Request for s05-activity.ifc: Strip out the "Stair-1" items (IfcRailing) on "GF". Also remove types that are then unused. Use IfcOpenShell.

First a look at what the model holds.

```python
import ifcopenshell
import ifcopenshell.util.element

model = ifcopenshell.open("s05-activity.ifc")
print(model.schema)
storey = next(s for s in model.by_type("IfcBuildingStorey") if s.Name == "GF")
railings = [e for e in ifcopenshell.util.element.get_decomposition(storey) if e.is_a("IfcRailing")]
seen = {}
for e in railings:
    element_type = ifcopenshell.util.element.get_type(e)
    name = element_type.Name if element_type not in (None, e) else None
    seen[name] = seen.get(name, 0) + 1
for name, count in sorted(seen.items(), key=str):
    print(count, "x", name)
```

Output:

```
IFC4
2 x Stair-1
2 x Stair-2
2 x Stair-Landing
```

```python
import ifcopenshell
import ifcopenshell.api.root
import ifcopenshell.util.element

model = ifcopenshell.open("s05-activity.ifc")

storey = next(s for s in model.by_type("IfcBuildingStorey") if s.Name == "GF")
railings = [e for e in ifcopenshell.util.element.get_decomposition(storey) if e.is_a("IfcRailing")]
targets = [e for e in railings if (t := ifcopenshell.util.element.get_type(e)) not in (None, e) and t.Name == "Stair-1"]
types = {ifcopenshell.util.element.get_type(e) for e in targets} - {None, *targets}

for e in targets:
    ifcopenshell.api.root.remove_product(model, product=e)
print(len(targets), "removed")

unused = [t for t in types if not ifcopenshell.util.element.get_types(t)]
for t in unused:
    ifcopenshell.api.root.remove_product(model, product=t)
print(len(unused), "unused types removed")

model.write("s05-activity-out.ifc")
```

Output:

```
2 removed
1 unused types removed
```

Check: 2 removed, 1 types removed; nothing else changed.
